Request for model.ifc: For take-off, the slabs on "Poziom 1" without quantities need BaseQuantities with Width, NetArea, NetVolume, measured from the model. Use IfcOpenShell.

First a look at what the model holds.

```python
import ifcopenshell
import ifcopenshell.util.element
import ifcopenshell.util.unit

model = ifcopenshell.open("model.ifc")
print(model.schema)
for unit_type in ("LENGTHUNIT", "AREAUNIT", "VOLUMEUNIT"):
    print(unit_type, ifcopenshell.util.unit.calculate_unit_scale(model, unit_type))
storey = next(s for s in model.by_type("IfcBuildingStorey") if s.Name == "Poziom 1")
slabs = [e for e in ifcopenshell.util.element.get_decomposition(storey) if e.is_a("IfcSlab")]
for e in sorted(slabs, key=lambda e: e.id()):
    print(e.id(), e.is_a(), e.Name, list(ifcopenshell.util.element.get_psets(e, qtos_only=True)), sep=" | ")
```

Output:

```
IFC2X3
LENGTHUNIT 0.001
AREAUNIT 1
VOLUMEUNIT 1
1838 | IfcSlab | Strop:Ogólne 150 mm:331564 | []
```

```python
import ifcopenshell
import ifcopenshell.api.pset
import ifcopenshell.geom
import ifcopenshell.util.element
import ifcopenshell.util.shape
import ifcopenshell.util.unit

model = ifcopenshell.open("model.ifc")
unit_scale = ifcopenshell.util.unit.calculate_unit_scale(model)
area_scale = ifcopenshell.util.unit.calculate_unit_scale(model, "AREAUNIT")
volume_scale = ifcopenshell.util.unit.calculate_unit_scale(model, "VOLUMEUNIT")
settings = ifcopenshell.geom.settings()

storey = next(s for s in model.by_type("IfcBuildingStorey") if s.Name == "Poziom 1")
slabs = [e for e in ifcopenshell.util.element.get_decomposition(storey) if e.is_a("IfcSlab")]

for e in sorted(slabs, key=lambda e: e.id()):
    if ifcopenshell.util.element.get_psets(e, qtos_only=True, should_inherit=False):
        continue
    # Geometry comes back in metres, in the element's own axes.
    shape = ifcopenshell.geom.create_shape(settings, e)
    values = {
        "Width": ifcopenshell.util.shape.get_z(shape.geometry) / unit_scale,
        "NetArea": ifcopenshell.util.shape.get_footprint_area(shape.geometry) / area_scale,
        "NetVolume": ifcopenshell.util.shape.get_volume(shape.geometry) / volume_scale,
    }
    qto = ifcopenshell.api.pset.add_qto(model, product=e, name="BaseQuantities")
    ifcopenshell.api.pset.edit_qto(model, qto=qto, properties=values)
    print(e.id(), {k: round(v, 3) for k, v in values.items()})

model.write("model_edited.ifc")
```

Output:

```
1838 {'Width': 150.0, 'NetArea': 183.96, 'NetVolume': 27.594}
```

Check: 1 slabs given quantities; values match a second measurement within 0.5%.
